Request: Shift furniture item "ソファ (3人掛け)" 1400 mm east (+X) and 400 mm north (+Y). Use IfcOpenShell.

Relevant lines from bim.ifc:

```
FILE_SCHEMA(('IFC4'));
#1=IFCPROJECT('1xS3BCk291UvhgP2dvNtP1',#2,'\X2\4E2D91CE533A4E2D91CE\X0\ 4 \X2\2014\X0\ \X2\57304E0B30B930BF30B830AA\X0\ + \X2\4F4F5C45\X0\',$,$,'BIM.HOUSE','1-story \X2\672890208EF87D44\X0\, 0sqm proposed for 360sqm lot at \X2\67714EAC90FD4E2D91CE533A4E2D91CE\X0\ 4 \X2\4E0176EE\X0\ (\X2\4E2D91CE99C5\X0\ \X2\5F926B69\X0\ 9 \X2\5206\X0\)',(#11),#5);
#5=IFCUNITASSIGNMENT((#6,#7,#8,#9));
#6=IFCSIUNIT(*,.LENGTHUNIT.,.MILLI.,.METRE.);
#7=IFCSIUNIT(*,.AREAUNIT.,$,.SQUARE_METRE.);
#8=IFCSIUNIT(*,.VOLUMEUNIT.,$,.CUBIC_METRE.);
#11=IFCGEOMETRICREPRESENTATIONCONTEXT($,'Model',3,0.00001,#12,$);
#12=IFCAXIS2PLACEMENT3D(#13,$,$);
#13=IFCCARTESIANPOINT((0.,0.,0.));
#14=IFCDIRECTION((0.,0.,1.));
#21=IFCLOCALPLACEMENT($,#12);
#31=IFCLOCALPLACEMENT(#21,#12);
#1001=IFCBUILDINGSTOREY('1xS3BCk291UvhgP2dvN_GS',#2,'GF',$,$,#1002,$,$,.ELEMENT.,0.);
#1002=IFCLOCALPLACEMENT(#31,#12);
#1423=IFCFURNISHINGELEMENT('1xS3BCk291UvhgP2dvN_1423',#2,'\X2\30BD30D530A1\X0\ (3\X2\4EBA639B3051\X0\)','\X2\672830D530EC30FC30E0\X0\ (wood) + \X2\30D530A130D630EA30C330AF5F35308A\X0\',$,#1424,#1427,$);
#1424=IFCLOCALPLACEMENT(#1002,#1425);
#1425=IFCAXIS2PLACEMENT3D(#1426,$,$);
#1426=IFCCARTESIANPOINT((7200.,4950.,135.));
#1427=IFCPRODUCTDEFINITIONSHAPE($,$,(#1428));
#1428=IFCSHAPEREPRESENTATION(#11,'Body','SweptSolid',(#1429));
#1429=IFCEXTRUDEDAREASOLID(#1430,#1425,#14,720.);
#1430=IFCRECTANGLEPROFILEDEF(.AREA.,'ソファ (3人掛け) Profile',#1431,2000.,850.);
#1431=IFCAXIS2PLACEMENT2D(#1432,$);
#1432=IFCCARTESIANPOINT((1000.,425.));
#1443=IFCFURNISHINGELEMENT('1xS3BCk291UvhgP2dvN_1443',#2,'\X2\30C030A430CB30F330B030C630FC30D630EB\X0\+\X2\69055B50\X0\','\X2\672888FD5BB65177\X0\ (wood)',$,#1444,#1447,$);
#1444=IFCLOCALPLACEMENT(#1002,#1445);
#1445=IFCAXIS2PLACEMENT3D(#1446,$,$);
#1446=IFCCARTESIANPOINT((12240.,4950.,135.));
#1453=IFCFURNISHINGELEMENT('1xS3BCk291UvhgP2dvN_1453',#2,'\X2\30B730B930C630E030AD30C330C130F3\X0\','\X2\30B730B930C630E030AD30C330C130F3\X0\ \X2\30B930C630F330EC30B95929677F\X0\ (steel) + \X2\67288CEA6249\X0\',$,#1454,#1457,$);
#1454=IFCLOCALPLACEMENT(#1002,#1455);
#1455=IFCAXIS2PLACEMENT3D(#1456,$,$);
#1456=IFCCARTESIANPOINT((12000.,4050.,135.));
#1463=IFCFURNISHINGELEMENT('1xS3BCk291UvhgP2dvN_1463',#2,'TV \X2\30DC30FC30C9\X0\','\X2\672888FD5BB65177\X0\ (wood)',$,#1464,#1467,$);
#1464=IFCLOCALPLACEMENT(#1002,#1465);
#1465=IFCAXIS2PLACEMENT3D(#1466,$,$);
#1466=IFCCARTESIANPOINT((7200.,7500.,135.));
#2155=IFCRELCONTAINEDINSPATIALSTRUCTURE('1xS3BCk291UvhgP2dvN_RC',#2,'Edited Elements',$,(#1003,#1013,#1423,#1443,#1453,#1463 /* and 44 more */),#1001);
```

```python
import ifcopenshell
import ifcopenshell.api.geometry
import ifcopenshell.util.placement

model = ifcopenshell.open("bim.ifc")

item = model.by_guid("1xS3BCk291UvhgP2dvN_1423")
matrix = ifcopenshell.util.placement.get_local_placement(item.ObjectPlacement)
matrix[0, 3] += 1400.0
matrix[1, 3] += 400.0
ifcopenshell.api.geometry.edit_object_placement(model, product=item, matrix=matrix, is_si=False)

print(ifcopenshell.util.placement.get_local_placement(item.ObjectPlacement).round(3) + 0.0)

model.write("bim_edited.ifc")
```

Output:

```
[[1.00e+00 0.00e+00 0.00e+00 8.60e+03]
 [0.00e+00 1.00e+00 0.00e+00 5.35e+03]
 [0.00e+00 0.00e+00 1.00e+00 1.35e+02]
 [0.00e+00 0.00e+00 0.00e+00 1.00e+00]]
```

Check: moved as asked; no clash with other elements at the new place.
